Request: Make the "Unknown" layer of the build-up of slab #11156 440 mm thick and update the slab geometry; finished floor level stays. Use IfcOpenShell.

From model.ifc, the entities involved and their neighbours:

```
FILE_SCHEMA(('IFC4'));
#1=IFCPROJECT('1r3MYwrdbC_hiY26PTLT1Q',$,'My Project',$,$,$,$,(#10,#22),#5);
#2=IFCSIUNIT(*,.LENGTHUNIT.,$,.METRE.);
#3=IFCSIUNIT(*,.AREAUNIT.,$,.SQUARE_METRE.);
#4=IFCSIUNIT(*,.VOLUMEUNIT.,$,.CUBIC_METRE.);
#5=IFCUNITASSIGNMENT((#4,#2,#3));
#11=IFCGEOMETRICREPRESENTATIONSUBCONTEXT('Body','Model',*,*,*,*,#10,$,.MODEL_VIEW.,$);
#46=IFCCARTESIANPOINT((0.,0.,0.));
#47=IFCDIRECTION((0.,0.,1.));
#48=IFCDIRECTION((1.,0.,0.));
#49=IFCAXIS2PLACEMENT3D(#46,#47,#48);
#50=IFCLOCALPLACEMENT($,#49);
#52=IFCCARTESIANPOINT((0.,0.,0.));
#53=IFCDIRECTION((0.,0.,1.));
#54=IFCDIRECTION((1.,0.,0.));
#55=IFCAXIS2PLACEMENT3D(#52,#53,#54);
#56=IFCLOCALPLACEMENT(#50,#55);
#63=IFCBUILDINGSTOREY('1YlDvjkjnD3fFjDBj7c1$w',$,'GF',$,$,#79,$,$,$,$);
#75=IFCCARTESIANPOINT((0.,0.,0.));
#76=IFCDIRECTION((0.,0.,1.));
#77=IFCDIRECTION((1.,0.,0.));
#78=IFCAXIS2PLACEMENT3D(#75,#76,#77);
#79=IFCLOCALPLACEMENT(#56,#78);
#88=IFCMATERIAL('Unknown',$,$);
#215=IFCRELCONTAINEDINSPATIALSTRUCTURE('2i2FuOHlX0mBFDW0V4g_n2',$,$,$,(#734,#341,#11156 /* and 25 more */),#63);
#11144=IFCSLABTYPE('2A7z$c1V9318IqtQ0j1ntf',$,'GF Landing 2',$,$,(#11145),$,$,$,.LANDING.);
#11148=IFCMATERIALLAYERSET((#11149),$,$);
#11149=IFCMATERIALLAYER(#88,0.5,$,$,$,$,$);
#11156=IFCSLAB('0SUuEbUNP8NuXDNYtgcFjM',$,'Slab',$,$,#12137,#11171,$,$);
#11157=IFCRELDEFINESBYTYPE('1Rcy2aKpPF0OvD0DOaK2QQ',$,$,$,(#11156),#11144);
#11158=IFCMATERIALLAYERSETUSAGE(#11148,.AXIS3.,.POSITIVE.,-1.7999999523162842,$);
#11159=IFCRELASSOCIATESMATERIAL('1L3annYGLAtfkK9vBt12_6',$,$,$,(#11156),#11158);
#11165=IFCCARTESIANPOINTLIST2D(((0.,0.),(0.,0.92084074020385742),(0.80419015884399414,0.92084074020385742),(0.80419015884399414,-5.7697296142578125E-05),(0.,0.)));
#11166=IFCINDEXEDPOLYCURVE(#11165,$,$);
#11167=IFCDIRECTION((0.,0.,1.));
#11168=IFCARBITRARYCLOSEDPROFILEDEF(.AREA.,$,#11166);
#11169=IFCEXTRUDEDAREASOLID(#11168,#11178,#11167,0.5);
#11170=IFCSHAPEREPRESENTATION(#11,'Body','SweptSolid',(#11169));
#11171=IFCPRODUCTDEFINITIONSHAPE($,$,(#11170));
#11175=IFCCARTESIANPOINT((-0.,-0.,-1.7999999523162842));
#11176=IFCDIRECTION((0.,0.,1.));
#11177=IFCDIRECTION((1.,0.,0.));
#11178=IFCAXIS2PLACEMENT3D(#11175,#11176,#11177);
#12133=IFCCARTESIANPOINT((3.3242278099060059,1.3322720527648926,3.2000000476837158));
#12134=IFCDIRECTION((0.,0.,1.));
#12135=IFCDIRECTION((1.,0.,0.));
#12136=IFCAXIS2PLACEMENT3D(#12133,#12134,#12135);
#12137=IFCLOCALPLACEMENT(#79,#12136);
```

```python
import ifcopenshell
import ifcopenshell.util.element
import ifcopenshell.util.representation
import ifcopenshell.util.unit

model = ifcopenshell.open("model.ifc")
unit_scale = ifcopenshell.util.unit.calculate_unit_scale(model)

layer_set = model.by_id(11148)
layer = next(l for l in layer_set.MaterialLayers if l.Material and l.Material.Name == "Unknown")
change = 0.44 / unit_scale - layer.LayerThickness
layer.LayerThickness += change

# Geometry does not follow the layer set by itself.
slabs = [e for e in ifcopenshell.util.element.get_elements_by_material(model, layer_set) if e.is_a("IfcSlab")]
for slab in sorted(slabs, key=lambda e: e.id()):
    body = ifcopenshell.util.representation.get_representation(slab, "Model", "Body")
    solid = body.Items[0]
    old_depth = solid.Depth
    solid.Depth += change
    # Extruded upwards: lower the start of the extrusion so the top stays.
    x, y, z = solid.Position.Location.Coordinates
    solid.Position.Location = model.createIfcCartesianPoint((x, y, z - change))
    print(slab.id(), f"{old_depth:g} -> {solid.Depth:g}")

# The layers are counted up from the underside, which has moved.
for usage in {ifcopenshell.util.element.get_material(slab) for slab in slabs}:
    usage.OffsetFromReferenceLine -= change

model.write("model_updated.ifc")
```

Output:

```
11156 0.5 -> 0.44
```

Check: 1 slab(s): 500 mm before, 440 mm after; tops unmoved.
